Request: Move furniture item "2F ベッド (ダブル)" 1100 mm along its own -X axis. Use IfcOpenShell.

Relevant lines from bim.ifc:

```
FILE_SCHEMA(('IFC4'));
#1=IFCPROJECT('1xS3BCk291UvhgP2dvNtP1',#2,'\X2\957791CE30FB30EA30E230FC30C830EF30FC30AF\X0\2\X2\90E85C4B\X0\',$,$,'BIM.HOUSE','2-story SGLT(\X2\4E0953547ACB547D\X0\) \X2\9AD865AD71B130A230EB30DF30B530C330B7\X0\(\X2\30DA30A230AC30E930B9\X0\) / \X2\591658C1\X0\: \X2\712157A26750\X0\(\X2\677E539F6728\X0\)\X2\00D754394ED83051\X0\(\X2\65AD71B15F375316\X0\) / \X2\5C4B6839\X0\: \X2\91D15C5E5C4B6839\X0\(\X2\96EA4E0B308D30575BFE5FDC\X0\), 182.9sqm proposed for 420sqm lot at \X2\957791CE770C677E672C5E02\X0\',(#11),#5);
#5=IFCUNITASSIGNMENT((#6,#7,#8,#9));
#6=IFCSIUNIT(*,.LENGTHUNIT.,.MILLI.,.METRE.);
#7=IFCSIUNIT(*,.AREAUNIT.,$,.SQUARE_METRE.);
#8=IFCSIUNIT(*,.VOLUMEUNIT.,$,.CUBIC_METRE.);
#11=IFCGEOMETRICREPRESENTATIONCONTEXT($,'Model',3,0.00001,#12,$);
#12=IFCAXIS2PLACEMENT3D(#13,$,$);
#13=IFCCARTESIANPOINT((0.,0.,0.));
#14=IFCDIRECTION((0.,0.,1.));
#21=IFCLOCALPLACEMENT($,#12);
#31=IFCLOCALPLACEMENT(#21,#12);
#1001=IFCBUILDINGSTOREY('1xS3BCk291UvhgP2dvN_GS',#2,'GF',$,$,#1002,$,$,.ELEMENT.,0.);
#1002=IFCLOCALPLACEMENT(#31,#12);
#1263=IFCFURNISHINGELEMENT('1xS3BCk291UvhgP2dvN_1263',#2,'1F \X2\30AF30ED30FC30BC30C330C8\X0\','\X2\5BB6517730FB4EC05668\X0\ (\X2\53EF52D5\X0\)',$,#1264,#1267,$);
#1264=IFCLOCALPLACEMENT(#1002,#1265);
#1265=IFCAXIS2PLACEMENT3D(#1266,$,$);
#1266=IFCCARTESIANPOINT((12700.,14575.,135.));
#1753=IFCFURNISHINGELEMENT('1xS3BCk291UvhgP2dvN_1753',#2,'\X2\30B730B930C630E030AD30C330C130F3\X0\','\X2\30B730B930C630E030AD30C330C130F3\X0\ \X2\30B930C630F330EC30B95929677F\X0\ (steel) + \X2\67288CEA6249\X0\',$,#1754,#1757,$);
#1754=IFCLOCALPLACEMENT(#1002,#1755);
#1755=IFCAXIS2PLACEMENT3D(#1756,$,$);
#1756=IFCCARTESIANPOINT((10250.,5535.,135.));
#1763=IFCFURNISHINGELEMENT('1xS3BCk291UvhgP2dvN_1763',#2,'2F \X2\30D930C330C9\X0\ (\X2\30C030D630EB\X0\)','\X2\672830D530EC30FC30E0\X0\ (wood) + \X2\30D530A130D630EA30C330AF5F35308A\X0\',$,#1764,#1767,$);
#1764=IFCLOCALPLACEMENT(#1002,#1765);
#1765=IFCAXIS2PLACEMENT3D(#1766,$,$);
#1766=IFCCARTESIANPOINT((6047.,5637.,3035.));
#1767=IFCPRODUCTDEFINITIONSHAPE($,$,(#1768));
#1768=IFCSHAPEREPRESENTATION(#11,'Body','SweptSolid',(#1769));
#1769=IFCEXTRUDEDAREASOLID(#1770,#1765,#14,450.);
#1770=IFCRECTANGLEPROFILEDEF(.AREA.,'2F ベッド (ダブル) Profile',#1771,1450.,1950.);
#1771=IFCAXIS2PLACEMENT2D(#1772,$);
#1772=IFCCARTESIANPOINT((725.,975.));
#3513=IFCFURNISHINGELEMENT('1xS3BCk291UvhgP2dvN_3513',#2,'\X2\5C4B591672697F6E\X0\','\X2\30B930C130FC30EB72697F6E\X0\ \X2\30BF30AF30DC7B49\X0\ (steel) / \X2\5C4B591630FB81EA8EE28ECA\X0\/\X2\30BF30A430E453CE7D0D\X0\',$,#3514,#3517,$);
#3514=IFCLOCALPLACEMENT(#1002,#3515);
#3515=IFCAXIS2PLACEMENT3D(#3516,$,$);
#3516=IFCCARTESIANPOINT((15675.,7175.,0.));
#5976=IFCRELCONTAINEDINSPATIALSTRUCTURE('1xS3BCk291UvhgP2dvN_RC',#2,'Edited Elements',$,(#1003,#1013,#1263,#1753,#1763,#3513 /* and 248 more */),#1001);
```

```python
import ifcopenshell
import ifcopenshell.api.geometry
import ifcopenshell.util.placement

model = ifcopenshell.open("bim.ifc")

item = model.by_guid("1xS3BCk291UvhgP2dvN_1763")
matrix = ifcopenshell.util.placement.get_local_placement(item.ObjectPlacement)
matrix[:3, 3] -= matrix[:3, 0] * 1100.0
ifcopenshell.api.geometry.edit_object_placement(model, product=item, matrix=matrix, is_si=False)

print(ifcopenshell.util.placement.get_local_placement(item.ObjectPlacement).round(3) + 0.0)

model.write("bim-out.ifc")
```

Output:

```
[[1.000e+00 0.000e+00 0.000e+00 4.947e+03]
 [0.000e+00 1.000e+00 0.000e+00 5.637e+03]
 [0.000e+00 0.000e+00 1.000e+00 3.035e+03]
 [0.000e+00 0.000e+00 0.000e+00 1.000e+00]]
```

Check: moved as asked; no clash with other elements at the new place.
